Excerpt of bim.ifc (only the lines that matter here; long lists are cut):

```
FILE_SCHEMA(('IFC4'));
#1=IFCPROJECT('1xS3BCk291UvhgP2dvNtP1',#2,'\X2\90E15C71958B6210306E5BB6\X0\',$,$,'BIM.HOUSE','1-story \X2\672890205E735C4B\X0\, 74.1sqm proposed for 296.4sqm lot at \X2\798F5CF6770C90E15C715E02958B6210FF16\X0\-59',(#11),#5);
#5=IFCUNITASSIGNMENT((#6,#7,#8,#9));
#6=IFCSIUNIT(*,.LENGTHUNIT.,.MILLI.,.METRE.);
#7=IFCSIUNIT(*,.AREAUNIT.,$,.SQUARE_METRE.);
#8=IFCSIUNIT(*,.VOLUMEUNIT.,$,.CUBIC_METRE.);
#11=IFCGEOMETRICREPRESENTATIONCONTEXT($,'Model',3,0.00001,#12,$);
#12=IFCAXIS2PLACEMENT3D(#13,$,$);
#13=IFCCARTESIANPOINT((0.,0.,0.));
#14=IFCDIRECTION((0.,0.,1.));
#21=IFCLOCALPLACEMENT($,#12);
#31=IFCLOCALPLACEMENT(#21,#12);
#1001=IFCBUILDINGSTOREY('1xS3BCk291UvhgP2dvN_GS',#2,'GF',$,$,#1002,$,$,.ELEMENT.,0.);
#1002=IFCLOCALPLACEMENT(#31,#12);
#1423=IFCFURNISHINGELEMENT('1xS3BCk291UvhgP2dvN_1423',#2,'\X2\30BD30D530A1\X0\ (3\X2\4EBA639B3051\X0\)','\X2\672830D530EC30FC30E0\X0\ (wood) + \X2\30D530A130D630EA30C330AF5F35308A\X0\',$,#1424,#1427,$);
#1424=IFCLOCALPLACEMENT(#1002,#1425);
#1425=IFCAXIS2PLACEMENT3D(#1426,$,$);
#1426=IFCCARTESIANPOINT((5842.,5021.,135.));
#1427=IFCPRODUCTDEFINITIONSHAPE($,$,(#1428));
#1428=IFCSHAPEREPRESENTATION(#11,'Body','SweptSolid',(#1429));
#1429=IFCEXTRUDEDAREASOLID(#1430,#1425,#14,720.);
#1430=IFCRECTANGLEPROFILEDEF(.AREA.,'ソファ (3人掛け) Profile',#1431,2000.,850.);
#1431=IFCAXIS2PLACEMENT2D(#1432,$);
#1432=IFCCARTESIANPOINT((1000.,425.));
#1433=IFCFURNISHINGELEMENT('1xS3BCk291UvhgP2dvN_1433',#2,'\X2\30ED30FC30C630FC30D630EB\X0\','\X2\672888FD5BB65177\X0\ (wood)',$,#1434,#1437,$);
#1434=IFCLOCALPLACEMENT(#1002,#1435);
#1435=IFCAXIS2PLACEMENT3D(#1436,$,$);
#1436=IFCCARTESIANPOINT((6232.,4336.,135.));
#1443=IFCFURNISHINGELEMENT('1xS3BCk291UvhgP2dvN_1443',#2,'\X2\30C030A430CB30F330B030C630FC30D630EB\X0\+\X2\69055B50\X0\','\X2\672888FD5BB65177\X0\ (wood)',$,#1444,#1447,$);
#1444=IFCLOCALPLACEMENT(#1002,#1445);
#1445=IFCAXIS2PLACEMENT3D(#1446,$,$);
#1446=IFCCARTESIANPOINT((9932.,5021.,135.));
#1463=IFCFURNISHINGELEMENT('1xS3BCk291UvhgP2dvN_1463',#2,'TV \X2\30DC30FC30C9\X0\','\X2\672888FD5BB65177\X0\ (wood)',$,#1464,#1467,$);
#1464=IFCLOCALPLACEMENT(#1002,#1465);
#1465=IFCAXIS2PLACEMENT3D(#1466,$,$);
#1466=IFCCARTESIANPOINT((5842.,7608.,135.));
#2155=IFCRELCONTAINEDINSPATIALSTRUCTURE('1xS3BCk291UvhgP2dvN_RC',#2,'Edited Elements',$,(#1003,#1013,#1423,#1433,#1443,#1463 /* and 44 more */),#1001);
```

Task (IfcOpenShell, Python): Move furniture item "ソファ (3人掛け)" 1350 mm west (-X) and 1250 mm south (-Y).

```python
import ifcopenshell
import ifcopenshell.api.geometry
import ifcopenshell.util.placement
import ifcopenshell.util.unit

model = ifcopenshell.open("bim.ifc")
unit_scale = ifcopenshell.util.unit.calculate_unit_scale(model)

item = model.by_guid("1xS3BCk291UvhgP2dvN_1423")
matrix = ifcopenshell.util.placement.get_local_placement(item.ObjectPlacement)
matrix[0, 3] -= 1.35 / unit_scale
matrix[1, 3] -= 1.25 / unit_scale
ifcopenshell.api.geometry.edit_object_placement(model, product=item, matrix=matrix, is_si=False)

print(ifcopenshell.util.placement.get_local_placement(item.ObjectPlacement).round(3) + 0.0)

model.write("bim_v2.ifc")
```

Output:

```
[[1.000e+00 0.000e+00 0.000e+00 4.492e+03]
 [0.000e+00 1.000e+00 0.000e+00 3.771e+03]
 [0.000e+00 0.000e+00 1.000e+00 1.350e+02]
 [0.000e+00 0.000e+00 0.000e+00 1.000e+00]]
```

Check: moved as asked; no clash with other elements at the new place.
